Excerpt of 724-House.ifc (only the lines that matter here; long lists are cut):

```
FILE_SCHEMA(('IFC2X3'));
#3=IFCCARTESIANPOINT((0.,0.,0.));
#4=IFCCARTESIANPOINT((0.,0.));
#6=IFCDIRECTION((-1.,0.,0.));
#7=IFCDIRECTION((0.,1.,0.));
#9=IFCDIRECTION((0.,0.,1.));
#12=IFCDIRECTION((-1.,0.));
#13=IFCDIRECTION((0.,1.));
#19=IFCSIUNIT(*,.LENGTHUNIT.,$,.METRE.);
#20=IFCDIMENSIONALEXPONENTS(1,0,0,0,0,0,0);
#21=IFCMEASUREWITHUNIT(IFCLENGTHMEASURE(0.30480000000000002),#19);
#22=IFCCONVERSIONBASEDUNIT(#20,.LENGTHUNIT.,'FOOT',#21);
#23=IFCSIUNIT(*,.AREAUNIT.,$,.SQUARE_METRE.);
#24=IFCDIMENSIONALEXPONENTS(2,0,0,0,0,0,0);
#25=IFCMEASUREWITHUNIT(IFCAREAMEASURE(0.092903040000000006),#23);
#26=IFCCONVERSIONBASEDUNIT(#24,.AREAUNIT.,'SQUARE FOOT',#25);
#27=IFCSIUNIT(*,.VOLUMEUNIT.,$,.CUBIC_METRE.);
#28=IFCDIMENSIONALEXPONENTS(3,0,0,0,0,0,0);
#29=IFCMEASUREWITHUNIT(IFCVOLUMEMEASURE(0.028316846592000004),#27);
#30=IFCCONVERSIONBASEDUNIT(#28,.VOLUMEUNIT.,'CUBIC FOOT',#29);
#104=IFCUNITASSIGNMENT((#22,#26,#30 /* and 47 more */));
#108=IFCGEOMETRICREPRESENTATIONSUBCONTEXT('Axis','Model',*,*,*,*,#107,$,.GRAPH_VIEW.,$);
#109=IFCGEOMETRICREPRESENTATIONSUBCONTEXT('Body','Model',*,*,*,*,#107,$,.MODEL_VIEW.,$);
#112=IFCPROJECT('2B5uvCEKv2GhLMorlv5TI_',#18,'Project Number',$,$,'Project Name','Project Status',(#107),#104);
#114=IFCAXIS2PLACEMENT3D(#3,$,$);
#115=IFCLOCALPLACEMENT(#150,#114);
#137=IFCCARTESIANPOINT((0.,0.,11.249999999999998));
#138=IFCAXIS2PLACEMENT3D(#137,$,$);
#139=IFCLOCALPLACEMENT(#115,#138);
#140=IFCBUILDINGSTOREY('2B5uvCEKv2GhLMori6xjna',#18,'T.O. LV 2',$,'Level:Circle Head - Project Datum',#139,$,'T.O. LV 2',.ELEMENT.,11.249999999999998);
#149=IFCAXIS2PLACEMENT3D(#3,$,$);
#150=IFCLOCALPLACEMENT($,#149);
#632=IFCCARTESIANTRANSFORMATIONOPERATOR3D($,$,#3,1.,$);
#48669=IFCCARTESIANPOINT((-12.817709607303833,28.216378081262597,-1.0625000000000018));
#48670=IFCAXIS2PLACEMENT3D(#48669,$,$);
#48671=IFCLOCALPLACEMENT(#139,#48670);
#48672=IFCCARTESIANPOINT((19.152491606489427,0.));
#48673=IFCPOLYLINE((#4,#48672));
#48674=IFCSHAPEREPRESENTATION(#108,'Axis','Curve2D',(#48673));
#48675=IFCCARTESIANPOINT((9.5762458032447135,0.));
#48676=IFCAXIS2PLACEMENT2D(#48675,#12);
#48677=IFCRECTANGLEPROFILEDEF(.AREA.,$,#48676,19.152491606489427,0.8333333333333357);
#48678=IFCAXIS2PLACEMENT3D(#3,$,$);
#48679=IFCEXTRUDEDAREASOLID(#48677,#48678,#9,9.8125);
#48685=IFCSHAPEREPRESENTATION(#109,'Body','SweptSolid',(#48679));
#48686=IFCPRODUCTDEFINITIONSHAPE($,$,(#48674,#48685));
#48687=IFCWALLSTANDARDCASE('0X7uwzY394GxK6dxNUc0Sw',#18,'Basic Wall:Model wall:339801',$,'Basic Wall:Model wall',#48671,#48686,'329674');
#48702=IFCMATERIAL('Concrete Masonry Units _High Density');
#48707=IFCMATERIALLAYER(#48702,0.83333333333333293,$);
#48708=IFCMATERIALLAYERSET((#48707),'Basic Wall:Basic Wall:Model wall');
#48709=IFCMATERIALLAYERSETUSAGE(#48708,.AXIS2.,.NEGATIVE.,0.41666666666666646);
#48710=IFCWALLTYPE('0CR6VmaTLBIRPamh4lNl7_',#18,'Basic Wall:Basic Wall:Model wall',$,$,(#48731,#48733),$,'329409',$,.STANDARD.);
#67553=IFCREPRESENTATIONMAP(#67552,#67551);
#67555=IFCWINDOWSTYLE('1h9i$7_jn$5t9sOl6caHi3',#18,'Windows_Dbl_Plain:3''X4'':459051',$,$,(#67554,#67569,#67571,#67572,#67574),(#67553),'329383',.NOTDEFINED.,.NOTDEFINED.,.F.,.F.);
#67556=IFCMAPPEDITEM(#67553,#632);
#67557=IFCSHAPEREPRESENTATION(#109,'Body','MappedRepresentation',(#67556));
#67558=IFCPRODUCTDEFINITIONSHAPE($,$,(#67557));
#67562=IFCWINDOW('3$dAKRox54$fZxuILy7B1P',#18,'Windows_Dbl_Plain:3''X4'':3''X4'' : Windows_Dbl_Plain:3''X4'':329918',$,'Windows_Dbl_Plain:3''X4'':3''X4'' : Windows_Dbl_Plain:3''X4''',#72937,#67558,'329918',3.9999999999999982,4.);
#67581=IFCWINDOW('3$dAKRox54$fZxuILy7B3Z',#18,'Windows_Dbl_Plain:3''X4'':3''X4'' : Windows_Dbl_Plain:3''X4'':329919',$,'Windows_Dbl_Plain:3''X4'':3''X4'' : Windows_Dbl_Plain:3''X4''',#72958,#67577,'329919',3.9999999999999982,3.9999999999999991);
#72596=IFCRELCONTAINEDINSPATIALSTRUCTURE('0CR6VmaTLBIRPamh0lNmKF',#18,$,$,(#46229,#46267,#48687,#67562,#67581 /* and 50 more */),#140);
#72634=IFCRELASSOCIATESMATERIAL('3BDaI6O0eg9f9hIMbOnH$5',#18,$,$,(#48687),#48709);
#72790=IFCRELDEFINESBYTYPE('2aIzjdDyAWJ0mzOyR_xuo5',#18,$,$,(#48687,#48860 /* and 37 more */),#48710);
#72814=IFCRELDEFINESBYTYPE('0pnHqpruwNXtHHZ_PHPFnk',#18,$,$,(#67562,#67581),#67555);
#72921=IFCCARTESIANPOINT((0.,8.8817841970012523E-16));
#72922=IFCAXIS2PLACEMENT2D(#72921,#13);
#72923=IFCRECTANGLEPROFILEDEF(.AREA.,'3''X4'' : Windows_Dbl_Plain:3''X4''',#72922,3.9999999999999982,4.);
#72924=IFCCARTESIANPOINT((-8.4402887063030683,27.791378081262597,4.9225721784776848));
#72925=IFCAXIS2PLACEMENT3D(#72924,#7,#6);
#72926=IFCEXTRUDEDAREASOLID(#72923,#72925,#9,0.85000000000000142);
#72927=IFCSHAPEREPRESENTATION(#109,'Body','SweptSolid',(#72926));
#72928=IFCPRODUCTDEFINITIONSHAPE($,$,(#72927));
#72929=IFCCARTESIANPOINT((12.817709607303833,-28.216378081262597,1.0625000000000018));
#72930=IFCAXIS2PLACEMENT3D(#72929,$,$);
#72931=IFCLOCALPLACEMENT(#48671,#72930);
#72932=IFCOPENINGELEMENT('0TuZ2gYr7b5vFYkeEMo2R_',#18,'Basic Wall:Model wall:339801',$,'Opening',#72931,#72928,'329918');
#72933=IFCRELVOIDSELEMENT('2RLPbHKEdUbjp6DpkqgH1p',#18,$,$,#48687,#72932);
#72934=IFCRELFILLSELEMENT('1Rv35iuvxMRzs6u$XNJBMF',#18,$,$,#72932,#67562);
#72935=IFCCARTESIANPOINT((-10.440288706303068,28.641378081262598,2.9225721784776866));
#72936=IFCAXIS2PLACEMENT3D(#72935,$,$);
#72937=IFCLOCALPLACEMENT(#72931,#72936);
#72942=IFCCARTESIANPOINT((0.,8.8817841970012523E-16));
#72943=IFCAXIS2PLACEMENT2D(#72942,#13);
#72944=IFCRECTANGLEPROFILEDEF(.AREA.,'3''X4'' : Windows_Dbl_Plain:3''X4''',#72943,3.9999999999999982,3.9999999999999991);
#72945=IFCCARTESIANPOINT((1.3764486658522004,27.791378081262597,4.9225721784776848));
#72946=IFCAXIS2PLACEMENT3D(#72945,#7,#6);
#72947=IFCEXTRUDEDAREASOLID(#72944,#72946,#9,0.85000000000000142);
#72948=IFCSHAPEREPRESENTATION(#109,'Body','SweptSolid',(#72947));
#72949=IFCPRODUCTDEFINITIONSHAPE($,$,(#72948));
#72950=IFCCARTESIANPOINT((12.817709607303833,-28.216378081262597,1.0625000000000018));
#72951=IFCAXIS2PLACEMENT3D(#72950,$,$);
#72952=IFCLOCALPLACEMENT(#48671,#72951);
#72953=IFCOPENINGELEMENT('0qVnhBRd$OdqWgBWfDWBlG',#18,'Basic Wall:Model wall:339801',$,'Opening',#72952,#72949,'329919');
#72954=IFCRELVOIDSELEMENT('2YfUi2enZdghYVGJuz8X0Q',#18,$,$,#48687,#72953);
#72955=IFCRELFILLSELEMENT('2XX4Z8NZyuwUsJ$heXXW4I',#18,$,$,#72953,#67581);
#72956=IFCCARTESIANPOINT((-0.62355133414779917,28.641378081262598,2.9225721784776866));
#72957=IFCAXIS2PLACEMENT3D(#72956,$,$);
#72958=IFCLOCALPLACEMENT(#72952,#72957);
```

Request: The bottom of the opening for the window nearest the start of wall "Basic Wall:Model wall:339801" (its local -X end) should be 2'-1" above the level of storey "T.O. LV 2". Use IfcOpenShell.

```python
import numpy as np
import ifcopenshell
import ifcopenshell.api.geometry
import ifcopenshell.geom
import ifcopenshell.util.element
import ifcopenshell.util.placement
import ifcopenshell.util.shape
import ifcopenshell.util.unit

model = ifcopenshell.open("724-House.ifc")
unit_scale = ifcopenshell.util.unit.calculate_unit_scale(model)

window = model.by_id(67562)
opening = window.FillsVoids[0].RelatingOpeningElement
storey = ifcopenshell.util.element.get_container(window, ifc_class="IfcBuildingStorey")
level = ifcopenshell.util.placement.get_local_placement(storey.ObjectPlacement)[2, 3]

# The opening's origin need not be at the sill, so measure its lowest point.
shape = ifcopenshell.geom.create_shape(ifcopenshell.geom.settings(), opening)
bottom = ifcopenshell.util.shape.get_shape_bottom_elevation(shape, shape.geometry) / unit_scale
dz = level + 25 * 0.0254 / unit_scale - bottom

shift = np.array([0.0, 0.0, dz])
# The window is placed relative to its opening, so it follows when the opening moves.
matrix = ifcopenshell.util.placement.get_local_placement(opening.ObjectPlacement)
matrix[:3, 3] += shift
ifcopenshell.api.geometry.edit_object_placement(
    model, product=opening, matrix=matrix, is_si=False, should_transform_children=True
)

print(f"moved by {dz * unit_scale:+.3f} m")

model.write("724-House_v2.ifc")
```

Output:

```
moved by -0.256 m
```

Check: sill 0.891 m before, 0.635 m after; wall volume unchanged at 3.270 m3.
